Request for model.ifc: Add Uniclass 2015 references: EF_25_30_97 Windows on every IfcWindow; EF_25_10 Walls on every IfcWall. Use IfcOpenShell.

First a look at what the model holds.

```python
import ifcopenshell

model = ifcopenshell.open("model.ifc")
print(model.schema)
print("classifications:", [c.Name for c in model.by_type("IfcClassification")])
for ifc_class in ("IfcDoor", "IfcRoof", "IfcStair", "IfcWall", "IfcWindow"):
    print(ifc_class, len(model.by_type(ifc_class)))
```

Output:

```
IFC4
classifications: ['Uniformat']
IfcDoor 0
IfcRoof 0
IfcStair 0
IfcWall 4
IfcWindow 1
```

```python
import ifcopenshell
import ifcopenshell.api.classification

model = ifcopenshell.open("model.ifc")

system = ifcopenshell.api.classification.add_classification(model, classification="Uniclass 2015")

codes = {
    "IfcWindow": ("EF_25_30_97", "Windows"),
    "IfcWall": ("EF_25_10", "Walls"),
}
for ifc_class, (code, name) in codes.items():
    products = model.by_type(ifc_class)
    ifcopenshell.api.classification.add_reference(
        model, products=products, classification=system, identification=code, name=name
    )
    print(code, len(products))

model.write("model-out.ifc")
```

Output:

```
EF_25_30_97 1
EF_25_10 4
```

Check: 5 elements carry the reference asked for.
